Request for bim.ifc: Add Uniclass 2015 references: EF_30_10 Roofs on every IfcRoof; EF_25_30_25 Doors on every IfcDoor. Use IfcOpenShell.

First a look at what the model holds.

```python
import ifcopenshell

model = ifcopenshell.open("bim.ifc")
print(model.schema)
print("classifications:", [c.Name for c in model.by_type("IfcClassification")])
for ifc_class in ("IfcDoor", "IfcRoof", "IfcStair", "IfcWall", "IfcWindow"):
    print(ifc_class, len(model.by_type(ifc_class)))
```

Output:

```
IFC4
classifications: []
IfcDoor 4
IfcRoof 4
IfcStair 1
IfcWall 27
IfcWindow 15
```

```python
import ifcopenshell
import ifcopenshell.api.classification

model = ifcopenshell.open("bim.ifc")

system = ifcopenshell.api.classification.add_classification(model, classification="Uniclass 2015")

codes = {
    "IfcRoof": ("EF_30_10", "Roofs"),
    "IfcDoor": ("EF_25_30_25", "Doors"),
}
for ifc_class, (code, name) in codes.items():
    products = model.by_type(ifc_class)
    ifcopenshell.api.classification.add_reference(
        model, products=products, classification=system, identification=code, name=name
    )
    print(code, len(products))

model.write("bim_updated.ifc")
```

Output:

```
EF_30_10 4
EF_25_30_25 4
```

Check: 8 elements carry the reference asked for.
